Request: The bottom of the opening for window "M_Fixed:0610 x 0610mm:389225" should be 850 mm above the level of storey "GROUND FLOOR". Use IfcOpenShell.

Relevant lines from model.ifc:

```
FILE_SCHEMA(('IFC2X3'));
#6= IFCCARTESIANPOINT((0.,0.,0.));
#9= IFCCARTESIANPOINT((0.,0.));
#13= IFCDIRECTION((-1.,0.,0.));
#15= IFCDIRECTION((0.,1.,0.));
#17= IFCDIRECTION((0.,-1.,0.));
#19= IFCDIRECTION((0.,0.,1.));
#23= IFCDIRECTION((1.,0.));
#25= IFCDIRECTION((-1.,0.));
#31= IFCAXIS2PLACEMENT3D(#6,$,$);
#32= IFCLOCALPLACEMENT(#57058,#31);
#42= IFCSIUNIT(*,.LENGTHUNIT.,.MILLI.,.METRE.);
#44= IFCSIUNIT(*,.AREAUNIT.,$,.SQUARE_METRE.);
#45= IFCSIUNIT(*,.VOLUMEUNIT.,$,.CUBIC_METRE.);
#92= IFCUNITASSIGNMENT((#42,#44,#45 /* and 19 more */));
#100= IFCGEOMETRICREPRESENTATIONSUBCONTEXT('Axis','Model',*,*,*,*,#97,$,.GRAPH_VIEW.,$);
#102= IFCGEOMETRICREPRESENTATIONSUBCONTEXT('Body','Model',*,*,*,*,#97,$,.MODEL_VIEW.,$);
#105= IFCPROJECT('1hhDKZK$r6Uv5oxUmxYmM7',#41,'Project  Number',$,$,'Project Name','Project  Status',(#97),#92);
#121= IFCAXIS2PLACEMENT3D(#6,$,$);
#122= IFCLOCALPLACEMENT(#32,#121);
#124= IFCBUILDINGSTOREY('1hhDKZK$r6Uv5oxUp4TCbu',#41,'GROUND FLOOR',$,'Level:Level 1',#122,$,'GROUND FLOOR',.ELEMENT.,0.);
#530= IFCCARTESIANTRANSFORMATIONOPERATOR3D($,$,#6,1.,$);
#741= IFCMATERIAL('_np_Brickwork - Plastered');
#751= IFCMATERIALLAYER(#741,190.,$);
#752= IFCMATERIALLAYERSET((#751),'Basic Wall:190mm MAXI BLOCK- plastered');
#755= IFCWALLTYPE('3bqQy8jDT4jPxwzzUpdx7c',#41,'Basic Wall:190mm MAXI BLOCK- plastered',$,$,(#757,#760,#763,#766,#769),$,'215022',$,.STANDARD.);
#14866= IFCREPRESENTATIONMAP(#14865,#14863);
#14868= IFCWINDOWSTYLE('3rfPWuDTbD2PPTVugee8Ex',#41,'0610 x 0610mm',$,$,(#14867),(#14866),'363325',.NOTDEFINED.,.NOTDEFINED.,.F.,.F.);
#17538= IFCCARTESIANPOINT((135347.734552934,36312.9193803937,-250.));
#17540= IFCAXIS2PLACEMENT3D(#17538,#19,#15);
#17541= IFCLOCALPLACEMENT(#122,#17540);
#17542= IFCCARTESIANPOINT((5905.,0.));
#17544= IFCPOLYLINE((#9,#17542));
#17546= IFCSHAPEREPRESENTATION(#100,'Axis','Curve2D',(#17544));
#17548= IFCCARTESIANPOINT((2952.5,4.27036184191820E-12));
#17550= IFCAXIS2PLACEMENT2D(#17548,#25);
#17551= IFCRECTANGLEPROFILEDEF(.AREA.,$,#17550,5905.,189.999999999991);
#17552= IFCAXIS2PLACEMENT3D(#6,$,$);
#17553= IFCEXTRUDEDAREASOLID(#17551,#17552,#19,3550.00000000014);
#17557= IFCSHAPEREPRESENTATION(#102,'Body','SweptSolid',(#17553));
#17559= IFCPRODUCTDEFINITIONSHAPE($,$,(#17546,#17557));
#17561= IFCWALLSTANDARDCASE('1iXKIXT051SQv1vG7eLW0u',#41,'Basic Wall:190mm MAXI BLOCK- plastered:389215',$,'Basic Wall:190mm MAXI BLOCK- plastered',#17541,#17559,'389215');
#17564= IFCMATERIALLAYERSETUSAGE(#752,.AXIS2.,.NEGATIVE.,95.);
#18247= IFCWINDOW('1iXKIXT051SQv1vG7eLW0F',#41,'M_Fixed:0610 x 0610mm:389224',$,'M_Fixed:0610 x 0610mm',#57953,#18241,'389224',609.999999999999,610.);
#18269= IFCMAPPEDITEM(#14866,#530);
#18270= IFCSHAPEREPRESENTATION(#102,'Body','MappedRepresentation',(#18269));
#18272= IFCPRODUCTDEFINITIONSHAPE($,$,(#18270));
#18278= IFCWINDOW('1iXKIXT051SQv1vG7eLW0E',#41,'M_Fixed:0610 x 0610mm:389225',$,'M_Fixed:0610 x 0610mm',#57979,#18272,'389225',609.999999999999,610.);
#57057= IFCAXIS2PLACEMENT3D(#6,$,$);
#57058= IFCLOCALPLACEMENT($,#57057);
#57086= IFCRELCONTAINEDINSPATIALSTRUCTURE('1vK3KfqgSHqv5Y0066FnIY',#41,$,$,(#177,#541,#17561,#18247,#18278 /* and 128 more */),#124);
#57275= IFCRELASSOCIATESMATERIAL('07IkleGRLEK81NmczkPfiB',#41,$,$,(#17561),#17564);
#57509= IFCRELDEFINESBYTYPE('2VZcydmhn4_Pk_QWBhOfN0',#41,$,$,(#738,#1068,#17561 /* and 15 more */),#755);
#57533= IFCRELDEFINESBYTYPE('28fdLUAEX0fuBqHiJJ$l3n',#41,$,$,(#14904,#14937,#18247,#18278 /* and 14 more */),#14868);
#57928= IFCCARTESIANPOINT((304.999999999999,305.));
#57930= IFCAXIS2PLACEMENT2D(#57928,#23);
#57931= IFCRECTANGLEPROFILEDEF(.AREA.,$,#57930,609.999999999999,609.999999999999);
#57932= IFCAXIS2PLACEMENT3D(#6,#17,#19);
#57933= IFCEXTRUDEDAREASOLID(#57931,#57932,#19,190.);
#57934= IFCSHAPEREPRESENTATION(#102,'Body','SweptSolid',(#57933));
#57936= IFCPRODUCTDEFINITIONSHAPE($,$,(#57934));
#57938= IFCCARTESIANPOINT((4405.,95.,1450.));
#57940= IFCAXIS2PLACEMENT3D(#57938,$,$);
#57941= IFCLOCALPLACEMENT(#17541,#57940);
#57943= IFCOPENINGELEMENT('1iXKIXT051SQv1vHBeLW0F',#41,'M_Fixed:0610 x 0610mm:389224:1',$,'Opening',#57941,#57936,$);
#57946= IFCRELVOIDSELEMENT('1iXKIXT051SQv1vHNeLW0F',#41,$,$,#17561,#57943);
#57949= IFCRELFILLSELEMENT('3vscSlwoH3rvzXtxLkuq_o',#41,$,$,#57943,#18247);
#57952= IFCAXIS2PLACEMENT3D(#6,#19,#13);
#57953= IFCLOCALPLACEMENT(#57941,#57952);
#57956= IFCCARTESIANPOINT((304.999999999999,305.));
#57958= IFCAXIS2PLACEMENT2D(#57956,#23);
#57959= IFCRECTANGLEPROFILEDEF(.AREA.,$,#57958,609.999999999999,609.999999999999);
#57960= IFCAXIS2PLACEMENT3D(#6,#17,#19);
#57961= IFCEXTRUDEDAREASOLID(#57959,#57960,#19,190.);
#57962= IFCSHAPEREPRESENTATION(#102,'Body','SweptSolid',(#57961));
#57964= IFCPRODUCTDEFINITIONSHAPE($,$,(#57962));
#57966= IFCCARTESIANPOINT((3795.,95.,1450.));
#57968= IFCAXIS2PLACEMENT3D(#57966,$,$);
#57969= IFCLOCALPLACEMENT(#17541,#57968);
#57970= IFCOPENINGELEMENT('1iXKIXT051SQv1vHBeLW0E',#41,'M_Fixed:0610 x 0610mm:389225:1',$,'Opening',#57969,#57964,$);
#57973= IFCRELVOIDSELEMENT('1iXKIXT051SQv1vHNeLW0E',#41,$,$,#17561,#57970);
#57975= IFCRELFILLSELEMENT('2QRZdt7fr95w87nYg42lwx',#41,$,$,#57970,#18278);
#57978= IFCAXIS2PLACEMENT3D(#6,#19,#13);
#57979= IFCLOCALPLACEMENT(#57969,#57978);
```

```python
import numpy as np
import ifcopenshell
import ifcopenshell.api.geometry
import ifcopenshell.geom
import ifcopenshell.util.element
import ifcopenshell.util.placement
import ifcopenshell.util.shape
import ifcopenshell.util.unit

model = ifcopenshell.open("model.ifc")
unit_scale = ifcopenshell.util.unit.calculate_unit_scale(model)

window = model.by_id(18278)
opening = window.FillsVoids[0].RelatingOpeningElement
storey = ifcopenshell.util.element.get_container(window, ifc_class="IfcBuildingStorey")
level = ifcopenshell.util.placement.get_local_placement(storey.ObjectPlacement)[2, 3]

# The opening's origin need not be at the sill, so measure its lowest point.
shape = ifcopenshell.geom.create_shape(ifcopenshell.geom.settings(), opening)
bottom = ifcopenshell.util.shape.get_shape_bottom_elevation(shape, shape.geometry) / unit_scale
dz = level + 0.85 / unit_scale - bottom

shift = np.array([0.0, 0.0, dz])
# The window is placed relative to its opening, so it follows when the opening moves.
matrix = ifcopenshell.util.placement.get_local_placement(opening.ObjectPlacement)
matrix[:3, 3] += shift
ifcopenshell.api.geometry.edit_object_placement(
    model, product=opening, matrix=matrix, is_si=False, should_transform_children=True
)

print(f"moved by {dz * unit_scale:+.3f} m")

model.write("model-out.ifc")
```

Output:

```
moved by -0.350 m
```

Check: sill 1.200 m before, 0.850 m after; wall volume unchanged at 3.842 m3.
